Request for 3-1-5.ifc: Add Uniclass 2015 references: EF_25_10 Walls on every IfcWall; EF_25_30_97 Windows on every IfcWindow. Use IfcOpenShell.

First a look at what the model holds.

```python
import ifcopenshell

model = ifcopenshell.open("3-1-5.ifc")
print(model.schema)
print("classifications:", [c.Name for c in model.by_type("IfcClassification")])
for ifc_class in ("IfcDoor", "IfcRoof", "IfcStair", "IfcWall", "IfcWindow"):
    print(ifc_class, len(model.by_type(ifc_class)))
```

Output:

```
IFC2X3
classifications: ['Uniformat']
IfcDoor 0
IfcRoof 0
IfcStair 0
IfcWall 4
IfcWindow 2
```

```python
import ifcopenshell
import ifcopenshell.api.classification

model = ifcopenshell.open("3-1-5.ifc")

# IFC2X3 requires Source and Edition and has no link from the project to the system.
system = model.create_entity("IfcClassification", Source="NBS", Edition="2015", Name="Uniclass 2015")

codes = {
    "IfcWall": ("EF_25_10", "Walls"),
    "IfcWindow": ("EF_25_30_97", "Windows"),
}
for ifc_class, (code, name) in codes.items():
    products = model.by_type(ifc_class)
    ifcopenshell.api.classification.add_reference(
        model, products=products, classification=system, identification=code, name=name
    )
    print(code, len(products))

model.write("3-1-5_edited.ifc")
```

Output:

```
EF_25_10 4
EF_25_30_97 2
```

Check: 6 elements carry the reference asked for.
